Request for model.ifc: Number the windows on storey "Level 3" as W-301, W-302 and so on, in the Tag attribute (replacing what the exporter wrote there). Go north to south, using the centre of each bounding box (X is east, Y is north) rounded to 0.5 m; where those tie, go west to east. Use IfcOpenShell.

First a look at what the model holds.

```python
import ifcopenshell
import ifcopenshell.util.element
import ifcopenshell.util.placement

model = ifcopenshell.open("model.ifc")
print(model.schema)
storey = next(s for s in model.by_type("IfcBuildingStorey") if s.Name == "Level 3")
windows = [e for e in ifcopenshell.util.element.get_decomposition(storey) if e.is_a("IfcWindow")]
for e in sorted(windows, key=lambda e: e.id()):
    origin = ifcopenshell.util.placement.get_local_placement(e.ObjectPlacement)[:3, 3]
    print(e.id(), e.Tag, e.Name, origin.round(2) + 0.0, sep=" | ")
```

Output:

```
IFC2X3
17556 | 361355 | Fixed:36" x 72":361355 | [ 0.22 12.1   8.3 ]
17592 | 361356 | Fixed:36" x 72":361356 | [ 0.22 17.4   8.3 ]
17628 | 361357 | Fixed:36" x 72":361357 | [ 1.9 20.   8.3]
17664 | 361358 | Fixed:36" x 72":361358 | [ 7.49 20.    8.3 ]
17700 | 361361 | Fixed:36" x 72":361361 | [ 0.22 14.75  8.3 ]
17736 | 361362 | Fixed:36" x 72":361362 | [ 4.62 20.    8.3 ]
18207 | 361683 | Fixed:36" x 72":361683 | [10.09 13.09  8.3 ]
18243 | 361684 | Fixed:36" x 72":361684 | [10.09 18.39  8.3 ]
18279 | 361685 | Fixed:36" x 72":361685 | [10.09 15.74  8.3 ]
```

```python
import ifcopenshell
import ifcopenshell.geom
import ifcopenshell.util.element
import ifcopenshell.util.shape

model = ifcopenshell.open("model.ifc")
settings = ifcopenshell.geom.settings()
settings.set("use-world-coords", True)


def centre(element):
    shape = ifcopenshell.geom.create_shape(settings, element)
    return ifcopenshell.util.shape.get_bbox_centroid(shape.geometry)


storey = next(s for s in model.by_type("IfcBuildingStorey") if s.Name == "Level 3")
windows = [e for e in ifcopenshell.util.element.get_decomposition(storey) if e.is_a("IfcWindow")]

# Insertion points can sit at a corner or the storey origin, so sort by the geometry (in metres).
centres = {e: centre(e) for e in windows}
windows.sort(key=lambda e: (-round(centres[e][1] / 0.5), centres[e][0]))

for i, e in enumerate(windows, start=1):
    number = f"W-3{i:02d}"
    e.Tag = number
    print(e.id(), number)

model.write("model_edited.ifc")
```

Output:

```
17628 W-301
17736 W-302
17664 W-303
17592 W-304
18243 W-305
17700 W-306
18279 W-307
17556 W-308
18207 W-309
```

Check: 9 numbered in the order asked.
